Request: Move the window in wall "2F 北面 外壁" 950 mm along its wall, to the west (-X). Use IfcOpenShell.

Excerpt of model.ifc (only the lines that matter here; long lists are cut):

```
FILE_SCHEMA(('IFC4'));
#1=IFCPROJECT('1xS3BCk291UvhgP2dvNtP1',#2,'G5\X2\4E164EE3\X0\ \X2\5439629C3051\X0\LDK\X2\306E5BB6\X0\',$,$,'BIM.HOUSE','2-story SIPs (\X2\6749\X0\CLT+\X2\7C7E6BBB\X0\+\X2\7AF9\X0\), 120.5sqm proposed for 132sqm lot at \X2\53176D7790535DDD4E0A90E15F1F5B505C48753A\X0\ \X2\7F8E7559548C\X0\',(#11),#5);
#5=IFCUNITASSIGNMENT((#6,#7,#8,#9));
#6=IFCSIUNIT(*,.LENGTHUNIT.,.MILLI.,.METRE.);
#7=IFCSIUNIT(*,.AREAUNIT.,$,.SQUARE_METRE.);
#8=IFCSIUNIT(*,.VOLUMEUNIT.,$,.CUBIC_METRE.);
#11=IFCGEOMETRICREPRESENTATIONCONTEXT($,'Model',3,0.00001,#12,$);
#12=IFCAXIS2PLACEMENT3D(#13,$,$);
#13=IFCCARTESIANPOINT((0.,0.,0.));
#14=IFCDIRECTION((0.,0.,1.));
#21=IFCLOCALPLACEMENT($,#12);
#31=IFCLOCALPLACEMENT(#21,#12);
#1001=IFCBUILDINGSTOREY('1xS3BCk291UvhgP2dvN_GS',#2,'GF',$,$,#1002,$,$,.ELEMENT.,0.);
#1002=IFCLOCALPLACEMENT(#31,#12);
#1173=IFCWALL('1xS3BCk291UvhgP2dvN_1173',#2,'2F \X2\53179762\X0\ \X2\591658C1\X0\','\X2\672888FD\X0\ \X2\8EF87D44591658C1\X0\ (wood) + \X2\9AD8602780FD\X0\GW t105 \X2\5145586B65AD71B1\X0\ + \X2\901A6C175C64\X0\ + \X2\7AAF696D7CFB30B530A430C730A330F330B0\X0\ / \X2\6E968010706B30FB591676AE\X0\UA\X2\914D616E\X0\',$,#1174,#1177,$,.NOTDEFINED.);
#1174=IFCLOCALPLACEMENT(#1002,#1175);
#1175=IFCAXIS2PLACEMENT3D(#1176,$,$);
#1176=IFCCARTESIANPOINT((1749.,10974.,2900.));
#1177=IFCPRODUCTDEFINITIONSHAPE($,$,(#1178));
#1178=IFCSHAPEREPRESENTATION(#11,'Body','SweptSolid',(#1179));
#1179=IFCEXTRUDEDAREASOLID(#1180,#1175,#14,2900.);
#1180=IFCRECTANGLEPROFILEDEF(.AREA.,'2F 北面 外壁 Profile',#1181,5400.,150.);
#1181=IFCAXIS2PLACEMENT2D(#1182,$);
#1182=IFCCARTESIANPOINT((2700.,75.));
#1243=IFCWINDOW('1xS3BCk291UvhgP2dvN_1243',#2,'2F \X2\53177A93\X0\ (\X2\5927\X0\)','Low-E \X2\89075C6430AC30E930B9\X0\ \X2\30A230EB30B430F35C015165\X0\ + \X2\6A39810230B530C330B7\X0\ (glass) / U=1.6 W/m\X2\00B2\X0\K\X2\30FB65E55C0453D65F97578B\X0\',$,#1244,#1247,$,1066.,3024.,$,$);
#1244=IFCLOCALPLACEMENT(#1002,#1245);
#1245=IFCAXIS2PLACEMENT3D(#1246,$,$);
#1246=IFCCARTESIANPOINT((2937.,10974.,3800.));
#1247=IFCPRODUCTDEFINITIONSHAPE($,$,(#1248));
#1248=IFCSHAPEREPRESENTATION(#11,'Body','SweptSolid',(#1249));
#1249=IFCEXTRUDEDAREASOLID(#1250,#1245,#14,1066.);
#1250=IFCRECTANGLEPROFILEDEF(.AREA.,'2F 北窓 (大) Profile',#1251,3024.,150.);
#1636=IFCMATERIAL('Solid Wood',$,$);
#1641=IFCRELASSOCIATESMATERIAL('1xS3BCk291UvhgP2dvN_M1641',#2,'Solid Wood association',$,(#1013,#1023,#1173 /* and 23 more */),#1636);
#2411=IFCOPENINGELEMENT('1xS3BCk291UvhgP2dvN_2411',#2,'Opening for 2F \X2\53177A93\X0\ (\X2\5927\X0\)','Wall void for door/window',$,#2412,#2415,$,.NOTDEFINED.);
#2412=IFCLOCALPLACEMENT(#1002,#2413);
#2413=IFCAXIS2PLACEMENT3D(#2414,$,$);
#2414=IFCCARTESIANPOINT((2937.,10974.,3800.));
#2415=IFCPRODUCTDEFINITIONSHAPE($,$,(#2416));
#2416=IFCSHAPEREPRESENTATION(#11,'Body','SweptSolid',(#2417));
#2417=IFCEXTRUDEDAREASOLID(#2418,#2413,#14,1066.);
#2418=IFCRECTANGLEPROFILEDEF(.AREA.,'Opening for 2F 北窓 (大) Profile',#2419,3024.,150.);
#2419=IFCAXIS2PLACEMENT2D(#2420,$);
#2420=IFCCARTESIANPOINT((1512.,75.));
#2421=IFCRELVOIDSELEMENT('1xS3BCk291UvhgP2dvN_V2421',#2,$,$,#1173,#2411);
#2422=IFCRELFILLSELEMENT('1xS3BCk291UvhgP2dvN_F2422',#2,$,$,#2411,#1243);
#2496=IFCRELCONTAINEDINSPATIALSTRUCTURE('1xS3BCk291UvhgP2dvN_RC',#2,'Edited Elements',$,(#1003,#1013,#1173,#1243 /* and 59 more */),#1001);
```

```python
import ifcopenshell
import ifcopenshell.api.geometry
import ifcopenshell.util.placement
import ifcopenshell.util.unit

model = ifcopenshell.open("model.ifc")
unit_scale = ifcopenshell.util.unit.calculate_unit_scale(model)

window = model.by_guid("1xS3BCk291UvhgP2dvN_1243")
opening = window.FillsVoids[0].RelatingOpeningElement
wall = opening.VoidsElements[0].RelatingBuildingElement

wall_matrix = ifcopenshell.util.placement.get_local_placement(wall.ObjectPlacement)
shift = wall_matrix[:3, 0] * -0.95 / unit_scale
before = ifcopenshell.util.placement.get_local_placement(window.ObjectPlacement)[:3, 3].copy()

# The window is not placed relative to its opening, so move both.
for product in (opening, window):
    matrix = ifcopenshell.util.placement.get_local_placement(product.ObjectPlacement)
    matrix[:3, 3] += shift
    ifcopenshell.api.geometry.edit_object_placement(model, product=product, matrix=matrix, is_si=False)

after = ifcopenshell.util.placement.get_local_placement(window.ObjectPlacement)[:3, 3]
print("window moved by", (after - before).round(3) + 0.0)

model.write("model-out.ifc")
```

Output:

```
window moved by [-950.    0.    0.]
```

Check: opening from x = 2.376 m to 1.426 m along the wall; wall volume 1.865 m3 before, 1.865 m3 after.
